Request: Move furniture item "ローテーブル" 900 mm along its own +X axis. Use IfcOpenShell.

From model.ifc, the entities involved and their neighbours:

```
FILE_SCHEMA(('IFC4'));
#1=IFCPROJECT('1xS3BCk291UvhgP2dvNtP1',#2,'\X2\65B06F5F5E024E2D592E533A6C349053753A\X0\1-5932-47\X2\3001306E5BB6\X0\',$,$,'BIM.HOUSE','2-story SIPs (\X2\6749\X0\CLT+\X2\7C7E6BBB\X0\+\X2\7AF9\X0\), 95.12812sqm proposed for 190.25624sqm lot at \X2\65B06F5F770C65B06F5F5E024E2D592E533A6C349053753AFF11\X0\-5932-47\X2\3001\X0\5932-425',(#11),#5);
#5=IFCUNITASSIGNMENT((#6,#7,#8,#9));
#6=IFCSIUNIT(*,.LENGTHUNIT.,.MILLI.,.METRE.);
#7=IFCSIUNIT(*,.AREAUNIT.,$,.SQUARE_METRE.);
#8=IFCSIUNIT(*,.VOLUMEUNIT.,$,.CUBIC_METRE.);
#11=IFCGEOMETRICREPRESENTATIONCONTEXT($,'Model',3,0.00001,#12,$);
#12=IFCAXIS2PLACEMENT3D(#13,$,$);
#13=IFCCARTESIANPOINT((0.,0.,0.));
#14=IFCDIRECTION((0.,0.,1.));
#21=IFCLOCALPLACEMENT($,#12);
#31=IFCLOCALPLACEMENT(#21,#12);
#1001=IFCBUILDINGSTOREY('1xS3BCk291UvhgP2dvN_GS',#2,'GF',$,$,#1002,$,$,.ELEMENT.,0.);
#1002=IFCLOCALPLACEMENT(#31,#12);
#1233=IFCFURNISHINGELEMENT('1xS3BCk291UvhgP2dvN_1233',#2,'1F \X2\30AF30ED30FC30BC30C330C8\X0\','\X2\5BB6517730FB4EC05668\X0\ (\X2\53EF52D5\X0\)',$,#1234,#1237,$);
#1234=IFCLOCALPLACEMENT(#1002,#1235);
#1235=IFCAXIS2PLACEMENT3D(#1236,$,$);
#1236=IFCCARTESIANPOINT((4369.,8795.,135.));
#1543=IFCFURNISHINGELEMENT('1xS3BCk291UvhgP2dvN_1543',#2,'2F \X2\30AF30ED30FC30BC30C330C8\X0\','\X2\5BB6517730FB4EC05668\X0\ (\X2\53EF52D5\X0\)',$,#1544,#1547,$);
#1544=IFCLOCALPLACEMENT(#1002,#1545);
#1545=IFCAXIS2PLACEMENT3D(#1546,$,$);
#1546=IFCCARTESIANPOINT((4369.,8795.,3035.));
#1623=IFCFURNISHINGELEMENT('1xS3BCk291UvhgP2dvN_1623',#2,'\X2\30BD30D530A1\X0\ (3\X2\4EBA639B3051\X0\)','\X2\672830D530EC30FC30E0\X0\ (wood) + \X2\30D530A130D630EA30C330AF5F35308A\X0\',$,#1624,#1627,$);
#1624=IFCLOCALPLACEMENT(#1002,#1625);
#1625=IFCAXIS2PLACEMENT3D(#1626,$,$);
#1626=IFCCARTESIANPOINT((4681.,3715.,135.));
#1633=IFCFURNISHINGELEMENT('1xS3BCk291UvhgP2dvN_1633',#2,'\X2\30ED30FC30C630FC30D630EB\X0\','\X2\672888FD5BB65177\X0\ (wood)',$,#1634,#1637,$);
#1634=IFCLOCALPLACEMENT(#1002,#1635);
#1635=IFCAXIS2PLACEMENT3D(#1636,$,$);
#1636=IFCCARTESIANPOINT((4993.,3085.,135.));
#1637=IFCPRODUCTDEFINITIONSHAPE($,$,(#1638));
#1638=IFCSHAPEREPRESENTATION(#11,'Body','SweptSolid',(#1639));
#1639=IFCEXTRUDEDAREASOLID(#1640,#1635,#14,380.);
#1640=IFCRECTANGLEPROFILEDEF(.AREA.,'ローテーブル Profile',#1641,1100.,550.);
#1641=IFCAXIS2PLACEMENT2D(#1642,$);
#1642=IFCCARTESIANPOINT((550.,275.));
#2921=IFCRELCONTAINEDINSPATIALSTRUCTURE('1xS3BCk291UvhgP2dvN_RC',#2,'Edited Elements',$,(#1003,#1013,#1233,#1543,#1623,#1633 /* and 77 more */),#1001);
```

```python
import ifcopenshell
import ifcopenshell.api.geometry
import ifcopenshell.util.placement
import ifcopenshell.util.unit

model = ifcopenshell.open("model.ifc")
unit_scale = ifcopenshell.util.unit.calculate_unit_scale(model)

item = model.by_id(1633)
matrix = ifcopenshell.util.placement.get_local_placement(item.ObjectPlacement)
matrix[:3, 3] += matrix[:3, 0] * 0.9 / unit_scale
ifcopenshell.api.geometry.edit_object_placement(model, product=item, matrix=matrix, is_si=False)

print(ifcopenshell.util.placement.get_local_placement(item.ObjectPlacement).round(3) + 0.0)

model.write("model_updated.ifc")
```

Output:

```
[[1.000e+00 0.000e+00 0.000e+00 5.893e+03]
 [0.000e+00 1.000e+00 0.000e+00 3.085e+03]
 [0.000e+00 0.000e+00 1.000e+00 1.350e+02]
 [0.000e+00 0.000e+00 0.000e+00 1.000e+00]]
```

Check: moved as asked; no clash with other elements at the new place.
